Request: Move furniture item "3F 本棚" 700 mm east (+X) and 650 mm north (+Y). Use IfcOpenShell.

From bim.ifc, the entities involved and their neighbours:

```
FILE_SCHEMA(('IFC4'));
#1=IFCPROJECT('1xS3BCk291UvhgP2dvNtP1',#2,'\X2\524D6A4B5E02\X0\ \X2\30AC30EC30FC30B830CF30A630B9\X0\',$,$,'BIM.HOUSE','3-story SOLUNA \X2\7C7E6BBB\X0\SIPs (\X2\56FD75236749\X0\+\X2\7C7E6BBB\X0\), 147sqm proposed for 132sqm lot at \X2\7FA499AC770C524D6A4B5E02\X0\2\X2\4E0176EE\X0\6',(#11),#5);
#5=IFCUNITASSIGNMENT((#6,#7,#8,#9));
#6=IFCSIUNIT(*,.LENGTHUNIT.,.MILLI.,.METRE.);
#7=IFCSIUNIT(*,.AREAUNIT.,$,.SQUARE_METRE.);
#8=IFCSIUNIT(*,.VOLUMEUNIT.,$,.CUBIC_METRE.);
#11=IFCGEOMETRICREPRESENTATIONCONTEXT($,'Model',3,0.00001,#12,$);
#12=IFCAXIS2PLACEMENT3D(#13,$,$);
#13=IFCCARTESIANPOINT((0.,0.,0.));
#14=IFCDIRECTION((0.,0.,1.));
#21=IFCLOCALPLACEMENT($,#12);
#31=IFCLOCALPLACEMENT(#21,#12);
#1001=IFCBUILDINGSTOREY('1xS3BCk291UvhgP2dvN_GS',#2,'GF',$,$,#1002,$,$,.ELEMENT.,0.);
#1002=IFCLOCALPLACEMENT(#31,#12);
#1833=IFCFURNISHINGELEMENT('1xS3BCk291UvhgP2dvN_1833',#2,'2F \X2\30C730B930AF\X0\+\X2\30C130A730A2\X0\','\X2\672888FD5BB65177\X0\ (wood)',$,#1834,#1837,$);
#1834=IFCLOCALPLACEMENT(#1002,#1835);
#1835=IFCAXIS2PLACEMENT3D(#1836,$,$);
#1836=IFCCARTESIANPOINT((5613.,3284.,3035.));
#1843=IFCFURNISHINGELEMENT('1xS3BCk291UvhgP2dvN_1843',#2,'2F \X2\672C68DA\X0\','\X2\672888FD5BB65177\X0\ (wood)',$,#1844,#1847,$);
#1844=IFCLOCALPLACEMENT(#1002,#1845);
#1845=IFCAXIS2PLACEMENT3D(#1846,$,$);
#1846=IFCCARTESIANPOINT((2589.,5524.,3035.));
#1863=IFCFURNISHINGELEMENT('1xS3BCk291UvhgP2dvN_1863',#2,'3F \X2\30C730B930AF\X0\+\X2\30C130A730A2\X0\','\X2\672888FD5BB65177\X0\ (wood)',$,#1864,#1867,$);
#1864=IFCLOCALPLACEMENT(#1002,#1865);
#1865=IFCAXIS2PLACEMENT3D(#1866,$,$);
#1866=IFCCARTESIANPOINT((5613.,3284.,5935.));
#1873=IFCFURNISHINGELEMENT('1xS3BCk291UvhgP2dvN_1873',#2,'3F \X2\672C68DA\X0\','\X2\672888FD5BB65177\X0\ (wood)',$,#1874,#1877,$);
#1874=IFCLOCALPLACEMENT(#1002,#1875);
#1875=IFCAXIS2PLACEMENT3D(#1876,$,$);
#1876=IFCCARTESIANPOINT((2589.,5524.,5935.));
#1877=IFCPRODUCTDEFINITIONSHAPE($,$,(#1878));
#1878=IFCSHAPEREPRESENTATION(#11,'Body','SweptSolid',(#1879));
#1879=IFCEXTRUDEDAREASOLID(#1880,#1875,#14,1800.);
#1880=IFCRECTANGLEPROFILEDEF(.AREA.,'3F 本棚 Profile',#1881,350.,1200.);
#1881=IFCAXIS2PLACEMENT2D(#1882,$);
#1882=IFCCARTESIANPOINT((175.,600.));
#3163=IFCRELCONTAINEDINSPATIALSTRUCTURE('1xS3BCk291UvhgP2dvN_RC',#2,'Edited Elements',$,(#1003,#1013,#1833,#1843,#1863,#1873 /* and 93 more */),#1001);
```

```python
import ifcopenshell
import ifcopenshell.api.geometry
import ifcopenshell.util.placement

model = ifcopenshell.open("bim.ifc")

item = model.by_guid("1xS3BCk291UvhgP2dvN_1873")
matrix = ifcopenshell.util.placement.get_local_placement(item.ObjectPlacement)
matrix[0, 3] += 700.0
matrix[1, 3] += 650.0
ifcopenshell.api.geometry.edit_object_placement(model, product=item, matrix=matrix, is_si=False)

print(ifcopenshell.util.placement.get_local_placement(item.ObjectPlacement).round(3) + 0.0)

model.write("bim_updated.ifc")
```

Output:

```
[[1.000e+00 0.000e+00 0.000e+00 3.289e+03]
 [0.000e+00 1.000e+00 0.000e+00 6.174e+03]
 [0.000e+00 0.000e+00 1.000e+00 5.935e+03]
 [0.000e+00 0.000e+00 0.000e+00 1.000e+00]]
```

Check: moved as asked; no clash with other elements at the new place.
